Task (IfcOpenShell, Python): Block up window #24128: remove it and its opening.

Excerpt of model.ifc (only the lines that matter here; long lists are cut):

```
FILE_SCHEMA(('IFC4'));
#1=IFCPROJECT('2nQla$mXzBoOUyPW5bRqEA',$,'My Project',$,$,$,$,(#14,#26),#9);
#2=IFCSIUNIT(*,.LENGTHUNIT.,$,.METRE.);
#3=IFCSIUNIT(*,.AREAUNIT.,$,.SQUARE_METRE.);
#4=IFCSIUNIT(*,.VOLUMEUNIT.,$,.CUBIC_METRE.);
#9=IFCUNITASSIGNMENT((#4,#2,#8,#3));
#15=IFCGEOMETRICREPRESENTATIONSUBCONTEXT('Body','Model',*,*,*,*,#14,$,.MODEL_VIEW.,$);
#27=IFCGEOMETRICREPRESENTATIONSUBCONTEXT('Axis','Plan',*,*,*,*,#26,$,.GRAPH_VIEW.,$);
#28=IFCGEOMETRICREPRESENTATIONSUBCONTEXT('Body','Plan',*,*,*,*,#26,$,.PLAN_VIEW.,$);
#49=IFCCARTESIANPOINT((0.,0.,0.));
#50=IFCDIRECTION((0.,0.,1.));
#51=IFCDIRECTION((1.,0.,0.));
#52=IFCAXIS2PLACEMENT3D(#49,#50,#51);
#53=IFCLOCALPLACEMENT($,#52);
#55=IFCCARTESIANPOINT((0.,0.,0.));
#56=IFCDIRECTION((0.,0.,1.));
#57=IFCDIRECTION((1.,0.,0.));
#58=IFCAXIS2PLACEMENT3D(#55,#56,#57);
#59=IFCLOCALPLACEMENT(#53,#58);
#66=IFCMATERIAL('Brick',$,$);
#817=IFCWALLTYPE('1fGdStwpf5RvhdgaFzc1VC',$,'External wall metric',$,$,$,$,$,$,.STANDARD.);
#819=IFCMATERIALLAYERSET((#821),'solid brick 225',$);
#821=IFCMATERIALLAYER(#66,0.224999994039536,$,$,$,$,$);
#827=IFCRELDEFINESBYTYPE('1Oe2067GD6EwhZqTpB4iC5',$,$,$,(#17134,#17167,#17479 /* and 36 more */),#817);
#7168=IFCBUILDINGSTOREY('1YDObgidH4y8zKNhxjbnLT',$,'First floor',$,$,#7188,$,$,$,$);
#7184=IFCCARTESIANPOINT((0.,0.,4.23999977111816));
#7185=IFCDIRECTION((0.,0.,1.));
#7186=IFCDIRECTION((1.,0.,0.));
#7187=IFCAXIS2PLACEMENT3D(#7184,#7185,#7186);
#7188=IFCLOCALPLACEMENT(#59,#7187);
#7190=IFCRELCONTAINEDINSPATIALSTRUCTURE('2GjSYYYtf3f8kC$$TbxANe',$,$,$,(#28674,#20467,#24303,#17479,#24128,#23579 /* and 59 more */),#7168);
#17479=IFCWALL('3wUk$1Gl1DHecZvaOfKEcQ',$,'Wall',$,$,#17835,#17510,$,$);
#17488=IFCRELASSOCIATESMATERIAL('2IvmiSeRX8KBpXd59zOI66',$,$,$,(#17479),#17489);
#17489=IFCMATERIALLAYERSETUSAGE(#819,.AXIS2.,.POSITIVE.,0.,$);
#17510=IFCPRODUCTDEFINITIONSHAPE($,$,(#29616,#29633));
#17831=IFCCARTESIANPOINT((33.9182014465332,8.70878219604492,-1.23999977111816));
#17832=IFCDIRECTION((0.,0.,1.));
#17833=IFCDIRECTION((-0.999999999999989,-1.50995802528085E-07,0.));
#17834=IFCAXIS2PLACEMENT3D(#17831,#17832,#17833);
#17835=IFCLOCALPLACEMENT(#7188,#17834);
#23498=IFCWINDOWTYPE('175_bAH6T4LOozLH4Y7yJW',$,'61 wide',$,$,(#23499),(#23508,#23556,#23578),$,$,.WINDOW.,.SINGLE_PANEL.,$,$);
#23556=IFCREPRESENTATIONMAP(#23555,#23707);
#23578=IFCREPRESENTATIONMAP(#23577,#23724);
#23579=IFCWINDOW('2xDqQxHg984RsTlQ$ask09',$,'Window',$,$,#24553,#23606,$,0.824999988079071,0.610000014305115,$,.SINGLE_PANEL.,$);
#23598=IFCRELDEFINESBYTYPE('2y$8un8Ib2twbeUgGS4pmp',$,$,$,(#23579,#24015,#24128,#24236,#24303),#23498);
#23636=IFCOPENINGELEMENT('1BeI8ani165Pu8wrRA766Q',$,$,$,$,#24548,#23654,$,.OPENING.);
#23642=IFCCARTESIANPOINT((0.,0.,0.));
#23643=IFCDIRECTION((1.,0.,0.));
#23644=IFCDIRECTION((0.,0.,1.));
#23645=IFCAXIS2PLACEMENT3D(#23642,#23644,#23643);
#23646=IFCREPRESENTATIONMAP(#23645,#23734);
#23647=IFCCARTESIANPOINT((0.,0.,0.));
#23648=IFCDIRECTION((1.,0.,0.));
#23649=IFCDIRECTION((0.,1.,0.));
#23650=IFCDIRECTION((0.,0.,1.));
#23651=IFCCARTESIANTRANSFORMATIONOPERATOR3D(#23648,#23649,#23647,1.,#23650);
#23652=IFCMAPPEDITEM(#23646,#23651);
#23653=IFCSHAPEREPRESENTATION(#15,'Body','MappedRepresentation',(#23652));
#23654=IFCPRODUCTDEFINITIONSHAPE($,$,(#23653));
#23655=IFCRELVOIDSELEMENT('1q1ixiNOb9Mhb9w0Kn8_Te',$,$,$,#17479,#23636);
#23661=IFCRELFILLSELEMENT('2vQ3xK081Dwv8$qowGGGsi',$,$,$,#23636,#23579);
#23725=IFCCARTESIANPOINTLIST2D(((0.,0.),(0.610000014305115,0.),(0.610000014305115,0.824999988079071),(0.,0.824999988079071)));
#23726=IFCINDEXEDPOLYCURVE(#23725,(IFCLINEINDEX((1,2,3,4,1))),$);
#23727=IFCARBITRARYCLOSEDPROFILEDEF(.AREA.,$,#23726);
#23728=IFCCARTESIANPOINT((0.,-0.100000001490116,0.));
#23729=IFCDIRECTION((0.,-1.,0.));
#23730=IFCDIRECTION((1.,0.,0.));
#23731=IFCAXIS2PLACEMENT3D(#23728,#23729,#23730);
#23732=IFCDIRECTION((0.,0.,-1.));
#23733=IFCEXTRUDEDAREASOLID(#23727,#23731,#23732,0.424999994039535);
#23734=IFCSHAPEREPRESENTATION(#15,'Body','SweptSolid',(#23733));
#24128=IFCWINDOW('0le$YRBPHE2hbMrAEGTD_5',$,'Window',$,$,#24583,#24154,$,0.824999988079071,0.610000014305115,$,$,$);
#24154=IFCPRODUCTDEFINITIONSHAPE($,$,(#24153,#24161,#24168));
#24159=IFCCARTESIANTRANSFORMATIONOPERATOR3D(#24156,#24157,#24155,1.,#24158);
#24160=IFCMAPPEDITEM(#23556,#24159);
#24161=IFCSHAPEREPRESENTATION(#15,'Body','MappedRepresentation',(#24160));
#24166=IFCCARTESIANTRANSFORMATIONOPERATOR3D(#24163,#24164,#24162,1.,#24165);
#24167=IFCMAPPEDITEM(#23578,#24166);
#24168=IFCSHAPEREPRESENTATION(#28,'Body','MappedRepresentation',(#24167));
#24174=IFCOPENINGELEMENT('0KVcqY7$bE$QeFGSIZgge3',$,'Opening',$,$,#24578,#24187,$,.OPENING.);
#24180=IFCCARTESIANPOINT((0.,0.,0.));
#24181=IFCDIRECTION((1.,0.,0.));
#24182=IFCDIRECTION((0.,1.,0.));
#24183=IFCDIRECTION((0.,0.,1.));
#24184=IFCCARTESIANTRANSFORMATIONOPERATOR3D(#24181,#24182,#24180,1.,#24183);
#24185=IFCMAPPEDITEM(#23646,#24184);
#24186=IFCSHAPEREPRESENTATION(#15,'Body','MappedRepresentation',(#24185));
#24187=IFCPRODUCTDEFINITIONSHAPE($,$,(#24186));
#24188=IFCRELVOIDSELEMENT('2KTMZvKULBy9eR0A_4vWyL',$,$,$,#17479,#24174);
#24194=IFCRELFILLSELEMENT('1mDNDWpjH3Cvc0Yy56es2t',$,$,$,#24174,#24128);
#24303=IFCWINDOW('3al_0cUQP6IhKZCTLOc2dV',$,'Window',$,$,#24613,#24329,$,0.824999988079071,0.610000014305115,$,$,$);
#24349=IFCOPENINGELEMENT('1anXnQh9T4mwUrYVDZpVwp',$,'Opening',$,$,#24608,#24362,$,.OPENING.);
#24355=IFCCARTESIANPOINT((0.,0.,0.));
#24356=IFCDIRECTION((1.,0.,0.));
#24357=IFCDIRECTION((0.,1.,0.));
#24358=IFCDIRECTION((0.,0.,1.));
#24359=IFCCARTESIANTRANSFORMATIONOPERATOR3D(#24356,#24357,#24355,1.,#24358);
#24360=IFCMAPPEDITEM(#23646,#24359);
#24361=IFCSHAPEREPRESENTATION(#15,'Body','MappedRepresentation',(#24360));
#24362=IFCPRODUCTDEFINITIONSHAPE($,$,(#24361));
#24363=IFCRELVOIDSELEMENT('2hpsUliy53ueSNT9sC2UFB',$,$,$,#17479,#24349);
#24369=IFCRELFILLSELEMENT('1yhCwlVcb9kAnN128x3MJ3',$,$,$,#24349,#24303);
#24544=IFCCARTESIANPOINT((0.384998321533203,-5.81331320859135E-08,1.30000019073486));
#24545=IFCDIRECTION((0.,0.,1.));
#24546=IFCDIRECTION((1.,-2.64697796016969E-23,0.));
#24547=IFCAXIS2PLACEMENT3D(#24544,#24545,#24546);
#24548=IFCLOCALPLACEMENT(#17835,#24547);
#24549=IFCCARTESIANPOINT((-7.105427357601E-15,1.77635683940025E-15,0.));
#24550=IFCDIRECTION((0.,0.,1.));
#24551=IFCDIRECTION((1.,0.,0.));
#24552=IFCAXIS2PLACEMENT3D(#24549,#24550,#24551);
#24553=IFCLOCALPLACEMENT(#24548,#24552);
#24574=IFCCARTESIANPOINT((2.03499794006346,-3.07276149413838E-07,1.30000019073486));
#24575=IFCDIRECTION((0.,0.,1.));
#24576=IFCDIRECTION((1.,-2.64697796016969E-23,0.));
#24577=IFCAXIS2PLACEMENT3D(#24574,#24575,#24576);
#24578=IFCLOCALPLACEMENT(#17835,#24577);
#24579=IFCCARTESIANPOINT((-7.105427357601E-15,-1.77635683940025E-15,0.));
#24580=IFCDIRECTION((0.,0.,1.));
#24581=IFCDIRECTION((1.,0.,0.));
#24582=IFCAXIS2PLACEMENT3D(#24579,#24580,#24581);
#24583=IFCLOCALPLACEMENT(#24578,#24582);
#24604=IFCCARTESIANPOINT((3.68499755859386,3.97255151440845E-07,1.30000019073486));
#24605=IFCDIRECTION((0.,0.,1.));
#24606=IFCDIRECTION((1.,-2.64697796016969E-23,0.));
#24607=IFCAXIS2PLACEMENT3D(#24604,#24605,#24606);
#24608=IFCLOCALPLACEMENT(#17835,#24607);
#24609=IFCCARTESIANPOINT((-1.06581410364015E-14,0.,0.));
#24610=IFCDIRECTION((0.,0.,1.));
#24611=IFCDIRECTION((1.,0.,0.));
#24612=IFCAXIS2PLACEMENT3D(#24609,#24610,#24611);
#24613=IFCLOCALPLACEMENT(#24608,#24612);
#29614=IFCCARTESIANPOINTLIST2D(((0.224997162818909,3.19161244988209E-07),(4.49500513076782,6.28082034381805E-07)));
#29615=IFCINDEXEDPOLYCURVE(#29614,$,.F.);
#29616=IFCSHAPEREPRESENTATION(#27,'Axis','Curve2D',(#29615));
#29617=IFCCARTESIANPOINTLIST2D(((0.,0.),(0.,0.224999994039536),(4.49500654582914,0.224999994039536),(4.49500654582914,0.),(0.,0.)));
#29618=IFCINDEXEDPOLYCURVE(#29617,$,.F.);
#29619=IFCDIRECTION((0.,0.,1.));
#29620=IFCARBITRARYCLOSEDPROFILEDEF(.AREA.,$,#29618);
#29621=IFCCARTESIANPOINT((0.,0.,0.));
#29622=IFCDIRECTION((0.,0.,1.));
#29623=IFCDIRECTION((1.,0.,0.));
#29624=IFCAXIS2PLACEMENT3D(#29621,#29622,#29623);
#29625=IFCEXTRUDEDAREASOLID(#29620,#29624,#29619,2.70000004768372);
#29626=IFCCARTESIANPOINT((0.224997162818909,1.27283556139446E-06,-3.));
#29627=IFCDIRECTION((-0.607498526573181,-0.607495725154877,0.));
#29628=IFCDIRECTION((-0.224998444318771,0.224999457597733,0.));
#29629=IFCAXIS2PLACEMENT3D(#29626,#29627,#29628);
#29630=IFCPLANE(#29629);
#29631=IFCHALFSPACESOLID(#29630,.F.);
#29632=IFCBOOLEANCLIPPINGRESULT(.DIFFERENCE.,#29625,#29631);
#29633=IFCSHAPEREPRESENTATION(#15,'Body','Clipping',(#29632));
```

```python
import ifcopenshell
import ifcopenshell.api.feature
import ifcopenshell.api.root
import ifcopenshell.geom
import ifcopenshell.util.shape

model = ifcopenshell.open("model.ifc")
settings = ifcopenshell.geom.settings()


def volume(element):
    """Net volume in cubic metres, openings subtracted."""
    shape = ifcopenshell.geom.create_shape(settings, element)
    return ifcopenshell.util.shape.get_volume(shape.geometry)


window = model.by_id(24128)
opening = window.FillsVoids[0].RelatingOpeningElement
wall = opening.VoidsElements[0].RelatingBuildingElement
before = volume(wall)

ifcopenshell.api.root.remove_product(model, product=window)
ifcopenshell.api.feature.remove_feature(model, feature=opening)

after = volume(wall)

print(f"wall volume {before:.3f} -> {after:.3f} m3")

model.write("model_rev.ifc")
```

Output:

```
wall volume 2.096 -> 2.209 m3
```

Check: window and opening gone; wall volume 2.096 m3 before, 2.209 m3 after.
